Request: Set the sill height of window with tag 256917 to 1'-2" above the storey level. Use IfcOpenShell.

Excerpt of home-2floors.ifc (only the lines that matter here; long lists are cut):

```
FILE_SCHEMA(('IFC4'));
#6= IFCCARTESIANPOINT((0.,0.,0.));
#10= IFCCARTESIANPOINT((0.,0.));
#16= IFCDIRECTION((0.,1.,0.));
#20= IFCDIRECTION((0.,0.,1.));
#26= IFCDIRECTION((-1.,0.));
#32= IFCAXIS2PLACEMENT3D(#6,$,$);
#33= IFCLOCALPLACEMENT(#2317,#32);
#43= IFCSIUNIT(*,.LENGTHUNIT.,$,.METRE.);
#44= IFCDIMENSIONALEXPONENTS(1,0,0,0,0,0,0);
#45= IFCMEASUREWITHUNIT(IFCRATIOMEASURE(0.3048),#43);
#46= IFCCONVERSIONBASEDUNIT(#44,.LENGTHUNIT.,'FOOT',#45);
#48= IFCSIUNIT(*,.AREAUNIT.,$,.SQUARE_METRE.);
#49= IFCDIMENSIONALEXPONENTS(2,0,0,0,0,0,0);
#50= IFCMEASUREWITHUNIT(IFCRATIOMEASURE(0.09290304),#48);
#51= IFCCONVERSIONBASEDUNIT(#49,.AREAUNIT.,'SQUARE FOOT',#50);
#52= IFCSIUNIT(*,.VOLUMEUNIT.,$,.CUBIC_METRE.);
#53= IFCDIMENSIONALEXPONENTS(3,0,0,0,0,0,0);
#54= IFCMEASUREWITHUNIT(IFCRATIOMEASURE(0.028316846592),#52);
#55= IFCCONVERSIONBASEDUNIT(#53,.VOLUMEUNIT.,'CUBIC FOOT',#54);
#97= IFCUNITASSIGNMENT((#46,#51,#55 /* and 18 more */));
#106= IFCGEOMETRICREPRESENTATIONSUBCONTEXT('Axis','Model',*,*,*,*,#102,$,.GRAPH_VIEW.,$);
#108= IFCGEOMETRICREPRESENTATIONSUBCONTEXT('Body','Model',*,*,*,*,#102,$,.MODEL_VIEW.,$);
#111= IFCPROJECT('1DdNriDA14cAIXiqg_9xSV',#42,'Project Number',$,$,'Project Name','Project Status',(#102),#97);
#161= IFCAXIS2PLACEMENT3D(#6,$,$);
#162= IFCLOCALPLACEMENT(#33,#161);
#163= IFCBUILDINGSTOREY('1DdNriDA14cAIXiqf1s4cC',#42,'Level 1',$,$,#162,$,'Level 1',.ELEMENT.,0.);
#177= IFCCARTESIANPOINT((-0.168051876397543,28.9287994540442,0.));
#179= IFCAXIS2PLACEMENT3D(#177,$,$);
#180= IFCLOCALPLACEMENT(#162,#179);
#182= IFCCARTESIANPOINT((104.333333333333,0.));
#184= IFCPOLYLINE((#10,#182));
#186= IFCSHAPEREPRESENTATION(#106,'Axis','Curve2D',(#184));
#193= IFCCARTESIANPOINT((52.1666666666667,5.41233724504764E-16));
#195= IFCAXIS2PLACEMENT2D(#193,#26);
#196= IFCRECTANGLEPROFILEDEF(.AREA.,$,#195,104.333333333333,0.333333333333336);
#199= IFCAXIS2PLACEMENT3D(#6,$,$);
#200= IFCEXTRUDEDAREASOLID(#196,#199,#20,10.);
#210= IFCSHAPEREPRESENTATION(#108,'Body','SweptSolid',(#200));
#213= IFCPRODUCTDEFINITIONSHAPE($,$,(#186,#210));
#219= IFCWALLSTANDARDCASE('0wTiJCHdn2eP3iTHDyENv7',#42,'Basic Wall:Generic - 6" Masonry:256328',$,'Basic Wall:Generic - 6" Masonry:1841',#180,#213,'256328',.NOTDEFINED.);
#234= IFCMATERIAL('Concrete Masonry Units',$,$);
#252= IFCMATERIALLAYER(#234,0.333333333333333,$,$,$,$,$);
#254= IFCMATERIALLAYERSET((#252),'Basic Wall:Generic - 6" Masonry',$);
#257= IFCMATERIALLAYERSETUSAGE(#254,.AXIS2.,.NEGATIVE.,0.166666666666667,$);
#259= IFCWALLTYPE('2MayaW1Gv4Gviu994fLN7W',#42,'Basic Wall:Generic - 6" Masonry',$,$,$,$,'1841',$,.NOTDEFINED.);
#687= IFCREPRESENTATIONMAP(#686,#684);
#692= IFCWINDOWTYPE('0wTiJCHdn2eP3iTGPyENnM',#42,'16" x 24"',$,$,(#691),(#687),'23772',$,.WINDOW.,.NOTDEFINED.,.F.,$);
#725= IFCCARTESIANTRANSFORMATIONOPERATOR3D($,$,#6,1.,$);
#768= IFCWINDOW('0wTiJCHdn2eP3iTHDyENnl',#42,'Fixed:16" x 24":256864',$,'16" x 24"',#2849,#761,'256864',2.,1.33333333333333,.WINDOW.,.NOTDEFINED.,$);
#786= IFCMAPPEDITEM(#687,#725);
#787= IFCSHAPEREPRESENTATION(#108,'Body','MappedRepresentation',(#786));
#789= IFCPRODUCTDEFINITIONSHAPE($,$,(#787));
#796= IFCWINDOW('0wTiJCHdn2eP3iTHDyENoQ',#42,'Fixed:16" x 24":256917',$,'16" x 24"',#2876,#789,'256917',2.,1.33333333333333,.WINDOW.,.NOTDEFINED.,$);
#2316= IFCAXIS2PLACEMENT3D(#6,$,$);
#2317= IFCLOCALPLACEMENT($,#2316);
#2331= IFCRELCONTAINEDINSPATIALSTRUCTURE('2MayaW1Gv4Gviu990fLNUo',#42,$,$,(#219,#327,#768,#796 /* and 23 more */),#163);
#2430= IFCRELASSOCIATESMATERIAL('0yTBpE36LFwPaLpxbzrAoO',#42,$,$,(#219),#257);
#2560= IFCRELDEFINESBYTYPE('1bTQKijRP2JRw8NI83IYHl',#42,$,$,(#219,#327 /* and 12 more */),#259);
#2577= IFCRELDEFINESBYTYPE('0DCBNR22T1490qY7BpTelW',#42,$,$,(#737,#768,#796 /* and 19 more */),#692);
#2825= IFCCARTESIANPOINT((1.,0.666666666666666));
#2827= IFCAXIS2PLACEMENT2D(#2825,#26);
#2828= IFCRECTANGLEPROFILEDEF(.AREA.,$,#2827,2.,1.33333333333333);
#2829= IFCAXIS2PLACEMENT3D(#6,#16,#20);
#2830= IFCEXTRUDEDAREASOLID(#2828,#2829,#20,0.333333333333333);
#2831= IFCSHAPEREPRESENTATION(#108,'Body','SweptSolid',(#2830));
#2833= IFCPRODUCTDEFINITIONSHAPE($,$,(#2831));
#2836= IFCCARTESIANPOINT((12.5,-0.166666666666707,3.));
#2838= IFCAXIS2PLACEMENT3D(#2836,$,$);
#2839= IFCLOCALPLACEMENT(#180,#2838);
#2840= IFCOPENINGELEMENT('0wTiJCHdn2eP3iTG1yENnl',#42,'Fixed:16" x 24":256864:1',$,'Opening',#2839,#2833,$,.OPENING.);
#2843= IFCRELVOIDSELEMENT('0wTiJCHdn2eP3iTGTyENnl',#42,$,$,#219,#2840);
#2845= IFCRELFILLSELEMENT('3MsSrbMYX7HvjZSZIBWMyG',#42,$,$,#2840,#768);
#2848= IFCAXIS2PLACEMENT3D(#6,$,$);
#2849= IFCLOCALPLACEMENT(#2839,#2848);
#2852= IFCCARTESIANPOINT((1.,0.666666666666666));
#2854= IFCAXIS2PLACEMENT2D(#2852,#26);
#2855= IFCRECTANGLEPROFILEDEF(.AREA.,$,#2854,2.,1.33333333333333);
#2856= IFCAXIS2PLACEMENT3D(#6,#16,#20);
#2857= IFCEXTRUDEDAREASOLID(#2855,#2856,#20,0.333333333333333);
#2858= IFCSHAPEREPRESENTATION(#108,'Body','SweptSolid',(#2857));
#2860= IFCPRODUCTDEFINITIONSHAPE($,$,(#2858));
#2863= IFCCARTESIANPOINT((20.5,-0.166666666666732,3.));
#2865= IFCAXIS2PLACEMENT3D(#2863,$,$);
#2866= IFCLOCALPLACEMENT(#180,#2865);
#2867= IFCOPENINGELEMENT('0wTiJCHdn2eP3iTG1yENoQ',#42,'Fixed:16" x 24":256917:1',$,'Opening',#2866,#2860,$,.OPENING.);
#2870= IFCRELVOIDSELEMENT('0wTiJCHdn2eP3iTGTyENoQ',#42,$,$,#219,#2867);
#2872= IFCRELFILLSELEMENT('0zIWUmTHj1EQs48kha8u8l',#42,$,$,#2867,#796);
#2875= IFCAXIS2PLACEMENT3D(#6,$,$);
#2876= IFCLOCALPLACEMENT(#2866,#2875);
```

```python
import numpy as np
import ifcopenshell
import ifcopenshell.api.geometry
import ifcopenshell.geom
import ifcopenshell.util.element
import ifcopenshell.util.placement
import ifcopenshell.util.shape
import ifcopenshell.util.unit

model = ifcopenshell.open("home-2floors.ifc")
unit_scale = ifcopenshell.util.unit.calculate_unit_scale(model)

window = model.by_guid("0wTiJCHdn2eP3iTHDyENoQ")
opening = window.FillsVoids[0].RelatingOpeningElement
storey = ifcopenshell.util.element.get_container(window, ifc_class="IfcBuildingStorey")
level = ifcopenshell.util.placement.get_local_placement(storey.ObjectPlacement)[2, 3]

# The opening's origin need not be at the sill, so measure its lowest point.
shape = ifcopenshell.geom.create_shape(ifcopenshell.geom.settings(), opening)
bottom = ifcopenshell.util.shape.get_shape_bottom_elevation(shape, shape.geometry) / unit_scale
dz = level + 14 * 0.0254 / unit_scale - bottom

shift = np.array([0.0, 0.0, dz])
# The window is placed relative to its opening, so it follows when the opening moves.
matrix = ifcopenshell.util.placement.get_local_placement(opening.ObjectPlacement)
matrix[:3, 3] += shift
ifcopenshell.api.geometry.edit_object_placement(
    model, product=opening, matrix=matrix, is_si=False, should_transform_children=True
)

print(f"moved by {dz * unit_scale:+.3f} m")

model.write("home-2floors-out.ifc")
```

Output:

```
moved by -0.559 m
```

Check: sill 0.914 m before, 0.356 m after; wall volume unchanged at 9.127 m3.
